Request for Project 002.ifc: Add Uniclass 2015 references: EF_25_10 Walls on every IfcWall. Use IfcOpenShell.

First a look at what the model holds.

```python
import ifcopenshell

model = ifcopenshell.open("Project 002.ifc")
print(model.schema)
print("classifications:", [c.Name for c in model.by_type("IfcClassification")])
for ifc_class in ("IfcDoor", "IfcRoof", "IfcStair", "IfcWall", "IfcWindow"):
    print(ifc_class, len(model.by_type(ifc_class)))
```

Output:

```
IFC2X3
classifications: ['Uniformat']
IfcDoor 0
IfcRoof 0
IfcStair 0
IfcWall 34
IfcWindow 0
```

```python
import ifcopenshell
import ifcopenshell.api.classification

model = ifcopenshell.open("Project 002.ifc")

# IFC2X3 requires Source and Edition and has no link from the project to the system.
system = model.create_entity("IfcClassification", Source="NBS", Edition="2015", Name="Uniclass 2015")

codes = {
    "IfcWall": ("EF_25_10", "Walls"),
}
for ifc_class, (code, name) in codes.items():
    products = model.by_type(ifc_class)
    ifcopenshell.api.classification.add_reference(
        model, products=products, classification=system, identification=code, name=name
    )
    print(code, len(products))

model.write("Project 002_rev.ifc")
```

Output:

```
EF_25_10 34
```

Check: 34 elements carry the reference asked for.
